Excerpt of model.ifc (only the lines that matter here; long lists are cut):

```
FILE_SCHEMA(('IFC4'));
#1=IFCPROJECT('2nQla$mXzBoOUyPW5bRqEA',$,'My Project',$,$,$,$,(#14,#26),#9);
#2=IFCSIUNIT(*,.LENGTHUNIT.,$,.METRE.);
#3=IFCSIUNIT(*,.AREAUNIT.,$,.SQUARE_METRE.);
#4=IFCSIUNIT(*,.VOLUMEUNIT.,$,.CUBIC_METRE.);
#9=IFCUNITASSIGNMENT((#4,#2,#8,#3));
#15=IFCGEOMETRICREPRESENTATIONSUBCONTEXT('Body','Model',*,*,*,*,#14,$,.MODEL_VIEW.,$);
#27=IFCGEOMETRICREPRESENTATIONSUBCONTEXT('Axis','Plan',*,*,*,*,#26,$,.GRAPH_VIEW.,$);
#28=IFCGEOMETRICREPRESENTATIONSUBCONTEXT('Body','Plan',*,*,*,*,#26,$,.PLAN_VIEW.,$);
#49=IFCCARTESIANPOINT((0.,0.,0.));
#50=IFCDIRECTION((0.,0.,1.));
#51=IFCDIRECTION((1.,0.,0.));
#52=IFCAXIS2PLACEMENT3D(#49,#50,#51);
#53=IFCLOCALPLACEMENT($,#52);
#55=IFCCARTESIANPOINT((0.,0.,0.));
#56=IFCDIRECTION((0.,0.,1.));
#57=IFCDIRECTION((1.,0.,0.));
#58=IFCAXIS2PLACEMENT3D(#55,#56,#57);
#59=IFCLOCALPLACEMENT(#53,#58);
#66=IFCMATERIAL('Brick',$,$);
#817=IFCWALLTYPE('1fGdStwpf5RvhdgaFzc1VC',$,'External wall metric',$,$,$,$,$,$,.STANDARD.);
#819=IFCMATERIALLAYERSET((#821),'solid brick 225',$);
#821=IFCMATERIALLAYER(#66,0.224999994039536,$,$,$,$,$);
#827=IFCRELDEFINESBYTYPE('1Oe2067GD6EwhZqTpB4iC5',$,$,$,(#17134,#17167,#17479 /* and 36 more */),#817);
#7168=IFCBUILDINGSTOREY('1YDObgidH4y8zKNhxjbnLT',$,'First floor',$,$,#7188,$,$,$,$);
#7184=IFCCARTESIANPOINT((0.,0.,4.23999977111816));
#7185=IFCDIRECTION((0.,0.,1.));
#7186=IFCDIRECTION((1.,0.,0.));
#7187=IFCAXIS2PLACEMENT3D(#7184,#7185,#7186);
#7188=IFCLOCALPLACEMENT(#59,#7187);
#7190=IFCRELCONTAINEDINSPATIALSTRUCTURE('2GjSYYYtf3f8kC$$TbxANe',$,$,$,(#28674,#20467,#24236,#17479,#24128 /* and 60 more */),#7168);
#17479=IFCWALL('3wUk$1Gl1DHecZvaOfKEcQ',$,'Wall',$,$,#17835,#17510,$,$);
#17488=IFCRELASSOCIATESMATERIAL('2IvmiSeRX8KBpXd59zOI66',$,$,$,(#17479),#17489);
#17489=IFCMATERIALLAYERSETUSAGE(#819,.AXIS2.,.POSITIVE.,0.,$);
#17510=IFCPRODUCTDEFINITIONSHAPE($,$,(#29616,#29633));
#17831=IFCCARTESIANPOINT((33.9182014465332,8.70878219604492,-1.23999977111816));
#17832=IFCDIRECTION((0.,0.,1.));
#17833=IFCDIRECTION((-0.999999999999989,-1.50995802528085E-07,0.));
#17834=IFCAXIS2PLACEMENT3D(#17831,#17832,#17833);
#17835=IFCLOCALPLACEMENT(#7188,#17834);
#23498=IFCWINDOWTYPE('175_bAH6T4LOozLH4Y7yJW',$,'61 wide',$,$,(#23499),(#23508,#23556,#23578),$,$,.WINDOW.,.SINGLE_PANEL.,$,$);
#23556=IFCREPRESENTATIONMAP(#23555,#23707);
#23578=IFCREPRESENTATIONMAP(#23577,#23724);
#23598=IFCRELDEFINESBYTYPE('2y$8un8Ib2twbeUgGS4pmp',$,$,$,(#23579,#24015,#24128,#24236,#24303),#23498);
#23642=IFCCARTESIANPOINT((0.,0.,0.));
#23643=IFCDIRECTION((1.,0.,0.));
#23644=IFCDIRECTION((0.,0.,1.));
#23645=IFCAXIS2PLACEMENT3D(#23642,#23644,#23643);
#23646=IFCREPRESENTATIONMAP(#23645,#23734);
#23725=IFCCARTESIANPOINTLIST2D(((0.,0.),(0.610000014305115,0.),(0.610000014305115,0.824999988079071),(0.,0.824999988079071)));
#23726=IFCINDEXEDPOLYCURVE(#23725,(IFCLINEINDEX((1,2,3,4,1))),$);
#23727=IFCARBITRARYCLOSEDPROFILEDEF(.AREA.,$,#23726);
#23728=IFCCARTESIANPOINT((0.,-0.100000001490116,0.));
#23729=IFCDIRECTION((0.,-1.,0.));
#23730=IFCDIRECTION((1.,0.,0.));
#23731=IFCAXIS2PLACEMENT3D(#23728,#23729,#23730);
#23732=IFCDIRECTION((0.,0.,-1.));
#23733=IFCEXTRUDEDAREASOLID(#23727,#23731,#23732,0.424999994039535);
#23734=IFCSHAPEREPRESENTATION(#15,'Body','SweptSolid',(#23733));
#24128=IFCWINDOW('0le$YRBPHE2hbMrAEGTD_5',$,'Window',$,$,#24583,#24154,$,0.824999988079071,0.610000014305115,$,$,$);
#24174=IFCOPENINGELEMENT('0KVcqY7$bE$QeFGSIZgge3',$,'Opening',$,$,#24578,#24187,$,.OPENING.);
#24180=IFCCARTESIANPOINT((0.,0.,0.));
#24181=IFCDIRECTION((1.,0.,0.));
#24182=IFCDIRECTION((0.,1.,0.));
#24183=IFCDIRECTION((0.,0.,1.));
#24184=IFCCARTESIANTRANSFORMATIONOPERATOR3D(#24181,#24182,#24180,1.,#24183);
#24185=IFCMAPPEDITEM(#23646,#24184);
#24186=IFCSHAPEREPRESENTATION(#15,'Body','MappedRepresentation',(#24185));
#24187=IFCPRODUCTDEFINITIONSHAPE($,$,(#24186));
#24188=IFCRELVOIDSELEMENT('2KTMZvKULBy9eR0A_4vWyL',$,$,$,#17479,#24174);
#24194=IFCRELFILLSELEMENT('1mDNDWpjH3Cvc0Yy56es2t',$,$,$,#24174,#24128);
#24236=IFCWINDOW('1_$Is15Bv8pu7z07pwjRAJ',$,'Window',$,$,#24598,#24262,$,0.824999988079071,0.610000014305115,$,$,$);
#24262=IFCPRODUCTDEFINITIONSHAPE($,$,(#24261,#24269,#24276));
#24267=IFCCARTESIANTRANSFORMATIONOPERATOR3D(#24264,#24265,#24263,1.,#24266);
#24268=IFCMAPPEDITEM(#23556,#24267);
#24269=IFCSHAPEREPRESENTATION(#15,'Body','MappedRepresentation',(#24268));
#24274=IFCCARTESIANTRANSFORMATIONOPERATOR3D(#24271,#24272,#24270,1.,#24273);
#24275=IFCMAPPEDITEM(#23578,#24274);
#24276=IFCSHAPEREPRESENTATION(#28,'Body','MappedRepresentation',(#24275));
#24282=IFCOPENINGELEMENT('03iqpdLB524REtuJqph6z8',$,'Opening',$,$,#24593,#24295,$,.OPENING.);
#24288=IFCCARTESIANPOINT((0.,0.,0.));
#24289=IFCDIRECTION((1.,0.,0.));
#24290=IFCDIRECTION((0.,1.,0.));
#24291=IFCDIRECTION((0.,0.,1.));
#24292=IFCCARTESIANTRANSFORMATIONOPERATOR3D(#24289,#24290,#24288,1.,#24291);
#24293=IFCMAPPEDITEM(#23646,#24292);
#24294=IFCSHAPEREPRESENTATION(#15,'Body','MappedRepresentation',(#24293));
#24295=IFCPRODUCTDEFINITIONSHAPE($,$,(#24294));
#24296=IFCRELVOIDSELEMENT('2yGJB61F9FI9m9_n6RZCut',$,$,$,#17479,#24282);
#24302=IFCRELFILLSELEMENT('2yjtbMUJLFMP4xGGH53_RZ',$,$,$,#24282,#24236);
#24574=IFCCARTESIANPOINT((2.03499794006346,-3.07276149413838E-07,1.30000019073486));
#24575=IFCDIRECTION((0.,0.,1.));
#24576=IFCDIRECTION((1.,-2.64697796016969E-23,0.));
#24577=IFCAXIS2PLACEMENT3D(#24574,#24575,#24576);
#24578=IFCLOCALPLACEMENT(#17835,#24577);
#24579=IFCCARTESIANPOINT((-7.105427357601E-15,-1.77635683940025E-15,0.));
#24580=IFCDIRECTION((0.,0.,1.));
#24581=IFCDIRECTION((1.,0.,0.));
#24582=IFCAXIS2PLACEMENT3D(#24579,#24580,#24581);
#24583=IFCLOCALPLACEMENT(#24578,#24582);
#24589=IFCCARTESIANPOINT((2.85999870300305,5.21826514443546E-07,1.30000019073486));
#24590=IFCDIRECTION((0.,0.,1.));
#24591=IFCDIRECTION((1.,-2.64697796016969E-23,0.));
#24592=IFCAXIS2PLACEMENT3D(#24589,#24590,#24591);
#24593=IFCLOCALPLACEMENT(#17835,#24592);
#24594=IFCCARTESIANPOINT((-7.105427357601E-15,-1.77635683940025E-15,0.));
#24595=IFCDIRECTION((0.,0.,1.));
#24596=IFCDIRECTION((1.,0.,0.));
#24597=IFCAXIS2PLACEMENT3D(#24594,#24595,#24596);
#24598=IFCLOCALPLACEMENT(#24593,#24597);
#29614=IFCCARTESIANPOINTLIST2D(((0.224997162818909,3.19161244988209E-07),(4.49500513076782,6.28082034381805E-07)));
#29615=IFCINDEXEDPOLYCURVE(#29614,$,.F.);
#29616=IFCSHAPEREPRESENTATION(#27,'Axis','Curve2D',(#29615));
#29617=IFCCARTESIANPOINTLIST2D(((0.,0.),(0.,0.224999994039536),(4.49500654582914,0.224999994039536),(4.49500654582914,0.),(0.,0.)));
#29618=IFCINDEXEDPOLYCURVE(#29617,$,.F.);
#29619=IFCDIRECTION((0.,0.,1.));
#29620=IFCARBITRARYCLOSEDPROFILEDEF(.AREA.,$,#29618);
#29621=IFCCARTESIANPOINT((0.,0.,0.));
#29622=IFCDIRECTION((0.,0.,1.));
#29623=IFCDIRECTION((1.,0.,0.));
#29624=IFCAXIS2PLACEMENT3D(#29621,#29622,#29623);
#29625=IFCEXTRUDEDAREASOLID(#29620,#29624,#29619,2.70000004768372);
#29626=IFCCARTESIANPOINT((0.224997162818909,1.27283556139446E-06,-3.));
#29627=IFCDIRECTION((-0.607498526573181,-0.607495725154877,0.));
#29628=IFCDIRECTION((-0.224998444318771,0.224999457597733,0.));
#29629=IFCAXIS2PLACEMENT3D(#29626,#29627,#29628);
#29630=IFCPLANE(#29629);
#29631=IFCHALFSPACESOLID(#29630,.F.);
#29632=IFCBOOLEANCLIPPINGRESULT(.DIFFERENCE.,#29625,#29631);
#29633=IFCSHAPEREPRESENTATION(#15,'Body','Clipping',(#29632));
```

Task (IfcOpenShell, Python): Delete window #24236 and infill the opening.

```python
import ifcopenshell
import ifcopenshell.api.feature
import ifcopenshell.api.root
import ifcopenshell.geom
import ifcopenshell.util.shape

model = ifcopenshell.open("model.ifc")
settings = ifcopenshell.geom.settings()


def volume(element):
    """Net volume in cubic metres, openings subtracted."""
    shape = ifcopenshell.geom.create_shape(settings, element)
    return ifcopenshell.util.shape.get_volume(shape.geometry)


window = model.by_id(24236)
opening = window.FillsVoids[0].RelatingOpeningElement
wall = opening.VoidsElements[0].RelatingBuildingElement
before = volume(wall)

ifcopenshell.api.root.remove_product(model, product=window)
ifcopenshell.api.feature.remove_feature(model, feature=opening)

after = volume(wall)

print(f"wall volume {before:.3f} -> {after:.3f} m3")

model.write("model_rev.ifc")
```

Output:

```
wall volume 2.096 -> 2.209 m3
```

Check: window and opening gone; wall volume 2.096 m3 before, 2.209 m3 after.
